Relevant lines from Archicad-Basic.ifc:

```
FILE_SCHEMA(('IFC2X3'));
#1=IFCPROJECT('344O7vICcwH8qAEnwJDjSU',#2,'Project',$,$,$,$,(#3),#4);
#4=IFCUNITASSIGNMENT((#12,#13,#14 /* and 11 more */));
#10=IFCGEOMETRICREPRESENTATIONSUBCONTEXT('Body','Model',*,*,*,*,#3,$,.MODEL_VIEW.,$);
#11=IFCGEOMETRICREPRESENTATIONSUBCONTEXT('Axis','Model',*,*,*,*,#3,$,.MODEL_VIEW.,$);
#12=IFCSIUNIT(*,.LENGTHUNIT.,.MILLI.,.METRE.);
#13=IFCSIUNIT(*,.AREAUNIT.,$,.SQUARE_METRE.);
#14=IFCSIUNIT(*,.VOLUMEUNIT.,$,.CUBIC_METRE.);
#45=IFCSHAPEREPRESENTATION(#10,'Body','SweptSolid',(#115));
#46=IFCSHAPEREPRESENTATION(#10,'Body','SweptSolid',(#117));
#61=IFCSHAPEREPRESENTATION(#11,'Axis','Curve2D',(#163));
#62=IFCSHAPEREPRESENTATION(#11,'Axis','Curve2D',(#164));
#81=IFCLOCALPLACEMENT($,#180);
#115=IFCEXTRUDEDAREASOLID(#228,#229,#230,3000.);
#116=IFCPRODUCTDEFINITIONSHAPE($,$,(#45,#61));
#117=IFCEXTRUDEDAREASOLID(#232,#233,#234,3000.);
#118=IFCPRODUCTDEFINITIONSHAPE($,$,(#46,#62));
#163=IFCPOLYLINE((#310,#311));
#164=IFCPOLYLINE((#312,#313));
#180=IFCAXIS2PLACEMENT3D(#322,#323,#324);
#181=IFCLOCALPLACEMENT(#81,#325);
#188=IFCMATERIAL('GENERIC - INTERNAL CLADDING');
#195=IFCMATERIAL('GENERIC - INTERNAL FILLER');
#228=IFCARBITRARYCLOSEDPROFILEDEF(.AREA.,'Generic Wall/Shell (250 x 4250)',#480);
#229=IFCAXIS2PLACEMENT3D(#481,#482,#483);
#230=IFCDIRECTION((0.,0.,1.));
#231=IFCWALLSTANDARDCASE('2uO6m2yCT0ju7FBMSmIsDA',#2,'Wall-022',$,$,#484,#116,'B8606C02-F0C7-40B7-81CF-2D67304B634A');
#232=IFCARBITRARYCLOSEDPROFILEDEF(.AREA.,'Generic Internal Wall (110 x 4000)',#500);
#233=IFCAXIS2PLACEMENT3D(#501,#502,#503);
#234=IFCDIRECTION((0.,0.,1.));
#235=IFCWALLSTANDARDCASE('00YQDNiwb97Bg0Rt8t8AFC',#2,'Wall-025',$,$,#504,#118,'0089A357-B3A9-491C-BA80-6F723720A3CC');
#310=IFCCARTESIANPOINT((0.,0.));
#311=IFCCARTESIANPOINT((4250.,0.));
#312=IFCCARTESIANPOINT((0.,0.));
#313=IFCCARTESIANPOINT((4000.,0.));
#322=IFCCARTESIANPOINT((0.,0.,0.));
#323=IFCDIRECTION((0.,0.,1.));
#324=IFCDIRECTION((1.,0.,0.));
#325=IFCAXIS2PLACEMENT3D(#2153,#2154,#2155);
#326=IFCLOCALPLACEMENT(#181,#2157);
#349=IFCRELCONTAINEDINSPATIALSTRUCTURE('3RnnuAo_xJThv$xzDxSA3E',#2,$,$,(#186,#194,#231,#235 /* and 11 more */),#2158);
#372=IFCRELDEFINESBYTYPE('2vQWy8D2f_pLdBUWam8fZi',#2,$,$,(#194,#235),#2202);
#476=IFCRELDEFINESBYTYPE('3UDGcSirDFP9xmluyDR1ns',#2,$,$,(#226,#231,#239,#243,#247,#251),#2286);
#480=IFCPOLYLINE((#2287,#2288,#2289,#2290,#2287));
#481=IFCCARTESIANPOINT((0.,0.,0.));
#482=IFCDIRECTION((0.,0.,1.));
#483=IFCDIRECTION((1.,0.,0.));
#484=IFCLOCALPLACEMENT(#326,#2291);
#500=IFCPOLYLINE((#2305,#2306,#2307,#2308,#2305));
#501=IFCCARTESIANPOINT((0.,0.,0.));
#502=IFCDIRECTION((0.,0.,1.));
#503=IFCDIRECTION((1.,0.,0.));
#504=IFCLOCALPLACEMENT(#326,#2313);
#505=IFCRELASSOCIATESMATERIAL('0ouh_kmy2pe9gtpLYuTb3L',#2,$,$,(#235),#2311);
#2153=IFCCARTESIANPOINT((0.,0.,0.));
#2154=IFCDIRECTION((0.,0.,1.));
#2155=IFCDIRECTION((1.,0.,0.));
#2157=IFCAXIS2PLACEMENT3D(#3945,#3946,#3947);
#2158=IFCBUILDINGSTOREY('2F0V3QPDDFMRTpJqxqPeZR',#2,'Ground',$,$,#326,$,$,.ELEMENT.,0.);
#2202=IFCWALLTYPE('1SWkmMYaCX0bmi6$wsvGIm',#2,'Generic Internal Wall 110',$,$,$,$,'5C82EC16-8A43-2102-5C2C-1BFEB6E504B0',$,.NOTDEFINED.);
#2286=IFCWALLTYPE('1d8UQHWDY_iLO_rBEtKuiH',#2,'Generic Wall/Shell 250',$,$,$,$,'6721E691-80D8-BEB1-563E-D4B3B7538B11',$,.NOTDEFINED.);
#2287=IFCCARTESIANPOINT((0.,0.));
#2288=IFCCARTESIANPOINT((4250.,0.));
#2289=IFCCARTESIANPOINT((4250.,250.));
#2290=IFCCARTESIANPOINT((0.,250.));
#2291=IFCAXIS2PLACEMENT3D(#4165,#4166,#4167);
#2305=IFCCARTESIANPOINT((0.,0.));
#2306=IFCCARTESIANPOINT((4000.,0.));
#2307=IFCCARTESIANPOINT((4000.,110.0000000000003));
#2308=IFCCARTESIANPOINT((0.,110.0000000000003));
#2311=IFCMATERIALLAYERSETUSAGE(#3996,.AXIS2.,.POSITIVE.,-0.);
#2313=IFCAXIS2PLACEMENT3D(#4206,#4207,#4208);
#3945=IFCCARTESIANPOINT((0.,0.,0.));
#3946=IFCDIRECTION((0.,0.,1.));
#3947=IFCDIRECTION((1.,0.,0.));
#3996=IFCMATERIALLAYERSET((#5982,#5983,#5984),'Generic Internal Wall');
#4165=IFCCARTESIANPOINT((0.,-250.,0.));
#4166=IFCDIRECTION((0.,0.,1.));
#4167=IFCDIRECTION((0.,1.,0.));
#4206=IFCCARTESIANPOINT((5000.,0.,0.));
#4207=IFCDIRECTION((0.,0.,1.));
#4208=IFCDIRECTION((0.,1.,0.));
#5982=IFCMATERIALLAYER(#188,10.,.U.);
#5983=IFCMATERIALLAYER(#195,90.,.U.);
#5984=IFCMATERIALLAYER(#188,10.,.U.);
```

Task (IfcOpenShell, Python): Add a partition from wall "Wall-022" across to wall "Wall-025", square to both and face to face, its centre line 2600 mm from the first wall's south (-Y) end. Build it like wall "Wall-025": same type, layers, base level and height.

```python
import numpy as np
import ifcopenshell
import ifcopenshell.api.geometry
import ifcopenshell.api.material
import ifcopenshell.api.pset
import ifcopenshell.api.root
import ifcopenshell.api.spatial
import ifcopenshell.api.type
import ifcopenshell.geom
import ifcopenshell.util.element
import ifcopenshell.util.placement
import ifcopenshell.util.representation
import ifcopenshell.util.shape
import ifcopenshell.util.unit

model = ifcopenshell.open("Archicad-Basic.ifc")
unit_scale = ifcopenshell.util.unit.calculate_unit_scale(model)
settings = ifcopenshell.geom.settings()
settings.set("use-world-coords", True)

start_wall = model.by_id(231)
end_wall = model.by_id(235)
like = model.by_guid("00YQDNiwb97Bg0Rt8t8AFC")
matrix = ifcopenshell.util.placement.get_local_placement(start_wall.ObjectPlacement)
matrix[:3, 3] *= unit_scale


def extent(element):
    """Bounding box in the first wall's axes, in metres."""
    shape = ifcopenshell.geom.create_shape(settings, element)
    points = (ifcopenshell.util.shape.get_vertices(shape.geometry) - matrix[:3, 3]) @ matrix[:3, :3]
    return points.min(axis=0), points.max(axis=0)


y_start = extent(start_wall)[0][1]
y_end = extent(end_wall)[1][1]
like_min, like_max = extent(like)
length, height = float(abs(y_end - y_start)), float(like_max[2] - like_min[2])
layer_set = ifcopenshell.util.element.get_material(like, should_skip_usage=True)
thickness = sum(layer.LayerThickness for layer in layer_set.MaterialLayers) * unit_scale

wall = ifcopenshell.api.root.create_entity(model, ifc_class="IfcWallStandardCase", name="New partition")
storey = ifcopenshell.util.element.get_container(like)
ifcopenshell.api.spatial.assign_container(model, products=[wall], relating_structure=storey)
ifcopenshell.api.type.assign_type(
    model, related_objects=[wall], relating_type=ifcopenshell.util.element.get_type(like), should_map_representations=False
)
rel = ifcopenshell.api.material.assign_material(
    model, products=[wall], type="IfcMaterialLayerSetUsage", material=layer_set
)
rel.RelatingMaterial.OffsetFromReferenceLine = -thickness / 2 / unit_scale
pset = ifcopenshell.api.pset.add_pset(model, product=wall, name="Pset_WallCommon")
ifcopenshell.api.pset.edit_pset(model, pset=pset, properties={"IsExternal": False, "LoadBearing": False})

# The axis runs down the middle of the wall.
axis = ifcopenshell.api.geometry.add_axis_representation(
    model, context=ifcopenshell.util.representation.get_context(model, "Model", "Axis"), axis=[(0.0, 0.0), (length, 0.0)]
)
body = ifcopenshell.api.geometry.add_wall_representation(
    model,
    context=ifcopenshell.util.representation.get_context(model, "Model", "Body", "MODEL_VIEW"),
    length=length,
    height=height,
    thickness=thickness,
    offset=-thickness / 2,
)
for representation in (axis, body):
    ifcopenshell.api.geometry.assign_representation(model, product=wall, representation=representation)

placement = matrix @ ifcopenshell.util.placement.rotation(-90, "Z")
placement[:, 3] = matrix @ np.array([extent(start_wall)[0][0] + 2.6, y_start, like_min[2], 1.0])
ifcopenshell.api.geometry.edit_object_placement(model, product=wall, matrix=placement)

print(f"partition {length:.3f} m long, {height:.3f} m high, {thickness:.3f} m thick")

model.write("Archicad-Basic_edited.ifc")
```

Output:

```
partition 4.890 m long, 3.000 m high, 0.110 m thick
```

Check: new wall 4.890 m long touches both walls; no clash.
